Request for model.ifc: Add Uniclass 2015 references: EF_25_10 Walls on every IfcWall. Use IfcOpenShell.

First a look at what the model holds.

```python
import ifcopenshell

model = ifcopenshell.open("model.ifc")
print(model.schema)
print("classifications:", [c.Name for c in model.by_type("IfcClassification")])
for ifc_class in ("IfcDoor", "IfcRoof", "IfcStair", "IfcWall", "IfcWindow"):
    print(ifc_class, len(model.by_type(ifc_class)))
```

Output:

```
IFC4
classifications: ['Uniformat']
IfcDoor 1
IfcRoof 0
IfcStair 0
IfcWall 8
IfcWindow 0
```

```python
import ifcopenshell
import ifcopenshell.api.classification

model = ifcopenshell.open("model.ifc")

system = ifcopenshell.api.classification.add_classification(model, classification="Uniclass 2015")

codes = {
    "IfcWall": ("EF_25_10", "Walls"),
}
for ifc_class, (code, name) in codes.items():
    products = model.by_type(ifc_class)
    ifcopenshell.api.classification.add_reference(
        model, products=products, classification=system, identification=code, name=name
    )
    print(code, len(products))

model.write("model_updated.ifc")
```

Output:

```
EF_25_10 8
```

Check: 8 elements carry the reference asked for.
